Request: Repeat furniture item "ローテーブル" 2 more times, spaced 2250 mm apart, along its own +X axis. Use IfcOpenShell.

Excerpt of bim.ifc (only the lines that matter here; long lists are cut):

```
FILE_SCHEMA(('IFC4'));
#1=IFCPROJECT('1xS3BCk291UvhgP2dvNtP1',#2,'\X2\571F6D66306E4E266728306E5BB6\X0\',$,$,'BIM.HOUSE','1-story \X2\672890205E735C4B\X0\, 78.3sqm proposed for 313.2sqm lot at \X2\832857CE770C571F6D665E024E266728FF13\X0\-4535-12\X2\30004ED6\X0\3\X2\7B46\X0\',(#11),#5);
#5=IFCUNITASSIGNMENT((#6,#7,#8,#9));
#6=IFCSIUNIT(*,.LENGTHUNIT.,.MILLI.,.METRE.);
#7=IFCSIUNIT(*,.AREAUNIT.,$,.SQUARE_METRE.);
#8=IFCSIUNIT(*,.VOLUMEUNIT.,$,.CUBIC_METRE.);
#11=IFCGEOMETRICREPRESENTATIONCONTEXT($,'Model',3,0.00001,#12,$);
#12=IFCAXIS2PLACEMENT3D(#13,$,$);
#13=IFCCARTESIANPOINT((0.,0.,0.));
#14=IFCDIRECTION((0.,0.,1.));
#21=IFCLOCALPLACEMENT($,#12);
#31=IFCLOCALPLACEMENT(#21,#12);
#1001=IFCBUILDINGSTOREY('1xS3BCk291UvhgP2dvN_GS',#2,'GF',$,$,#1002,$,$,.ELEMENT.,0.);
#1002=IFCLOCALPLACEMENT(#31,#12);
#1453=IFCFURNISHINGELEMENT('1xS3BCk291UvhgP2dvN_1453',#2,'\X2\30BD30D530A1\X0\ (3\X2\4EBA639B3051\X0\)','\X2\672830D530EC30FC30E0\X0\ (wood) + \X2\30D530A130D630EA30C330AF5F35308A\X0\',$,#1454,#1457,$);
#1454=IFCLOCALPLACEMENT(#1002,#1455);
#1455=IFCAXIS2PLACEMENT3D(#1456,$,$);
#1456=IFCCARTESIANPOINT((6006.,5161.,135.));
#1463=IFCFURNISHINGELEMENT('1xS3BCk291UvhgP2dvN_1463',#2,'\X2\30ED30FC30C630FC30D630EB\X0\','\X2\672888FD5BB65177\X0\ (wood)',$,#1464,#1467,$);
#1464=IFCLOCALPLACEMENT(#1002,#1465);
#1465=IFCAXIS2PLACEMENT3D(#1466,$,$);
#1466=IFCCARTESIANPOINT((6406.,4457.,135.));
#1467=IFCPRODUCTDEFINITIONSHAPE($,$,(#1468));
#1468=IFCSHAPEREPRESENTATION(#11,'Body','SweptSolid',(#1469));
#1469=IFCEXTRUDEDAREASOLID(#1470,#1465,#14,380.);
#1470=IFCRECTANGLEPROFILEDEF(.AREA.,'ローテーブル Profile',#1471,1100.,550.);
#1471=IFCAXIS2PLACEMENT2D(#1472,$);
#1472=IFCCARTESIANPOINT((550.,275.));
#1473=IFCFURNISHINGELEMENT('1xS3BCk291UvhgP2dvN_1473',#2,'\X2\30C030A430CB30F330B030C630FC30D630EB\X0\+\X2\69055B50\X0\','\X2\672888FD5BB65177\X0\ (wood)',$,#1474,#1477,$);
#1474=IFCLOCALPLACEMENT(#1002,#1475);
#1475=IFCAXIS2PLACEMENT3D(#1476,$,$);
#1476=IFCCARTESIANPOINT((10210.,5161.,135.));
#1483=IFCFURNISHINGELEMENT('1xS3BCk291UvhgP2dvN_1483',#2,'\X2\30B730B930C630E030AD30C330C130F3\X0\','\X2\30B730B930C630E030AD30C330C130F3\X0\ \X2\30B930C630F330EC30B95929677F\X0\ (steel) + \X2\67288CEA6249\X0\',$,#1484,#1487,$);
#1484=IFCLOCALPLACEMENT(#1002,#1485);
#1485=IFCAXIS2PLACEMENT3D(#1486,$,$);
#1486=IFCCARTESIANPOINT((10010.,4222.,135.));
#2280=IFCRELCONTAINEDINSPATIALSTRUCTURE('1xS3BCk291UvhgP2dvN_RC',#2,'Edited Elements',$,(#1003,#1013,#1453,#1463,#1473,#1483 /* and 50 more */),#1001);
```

```python
import ifcopenshell
import ifcopenshell.api.geometry
import ifcopenshell.api.root
import ifcopenshell.util.element
import ifcopenshell.util.placement

model = ifcopenshell.open("bim.ifc")


def reuse_history(source, copy):
    """copy_class also copies each property set's owner history, people and application; keep the originals."""
    for rel in copy.IsDefinedBy:
        if rel.is_a("IfcRelDefinesByProperties") and (history := rel.RelatingPropertyDefinition.OwnerHistory):
            rel.RelatingPropertyDefinition.OwnerHistory = source.OwnerHistory
            ifcopenshell.util.element.remove_deep2(model, history)


source = model.by_id(1463)
base = ifcopenshell.util.placement.get_local_placement(source.ObjectPlacement)
step = base[:3, 0] * 2250.0

for i in range(1, 3):
    copy = ifcopenshell.api.root.copy_class(model, product=source)
    copy.Representation = ifcopenshell.util.element.copy_deep(
        model, source.Representation, exclude=["IfcGeometricRepresentationContext", "IfcRepresentationMap"]
    )
    reuse_history(source, copy)
    matrix = base.copy()
    matrix[:3, 3] += i * step
    print("added at", matrix[:3, 3].round(3) + 0.0)
    ifcopenshell.api.geometry.edit_object_placement(model, product=copy, matrix=matrix, is_si=False)

model.write("bim_edited.ifc")
```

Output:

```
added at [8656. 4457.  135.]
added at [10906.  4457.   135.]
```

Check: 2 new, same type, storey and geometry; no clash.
